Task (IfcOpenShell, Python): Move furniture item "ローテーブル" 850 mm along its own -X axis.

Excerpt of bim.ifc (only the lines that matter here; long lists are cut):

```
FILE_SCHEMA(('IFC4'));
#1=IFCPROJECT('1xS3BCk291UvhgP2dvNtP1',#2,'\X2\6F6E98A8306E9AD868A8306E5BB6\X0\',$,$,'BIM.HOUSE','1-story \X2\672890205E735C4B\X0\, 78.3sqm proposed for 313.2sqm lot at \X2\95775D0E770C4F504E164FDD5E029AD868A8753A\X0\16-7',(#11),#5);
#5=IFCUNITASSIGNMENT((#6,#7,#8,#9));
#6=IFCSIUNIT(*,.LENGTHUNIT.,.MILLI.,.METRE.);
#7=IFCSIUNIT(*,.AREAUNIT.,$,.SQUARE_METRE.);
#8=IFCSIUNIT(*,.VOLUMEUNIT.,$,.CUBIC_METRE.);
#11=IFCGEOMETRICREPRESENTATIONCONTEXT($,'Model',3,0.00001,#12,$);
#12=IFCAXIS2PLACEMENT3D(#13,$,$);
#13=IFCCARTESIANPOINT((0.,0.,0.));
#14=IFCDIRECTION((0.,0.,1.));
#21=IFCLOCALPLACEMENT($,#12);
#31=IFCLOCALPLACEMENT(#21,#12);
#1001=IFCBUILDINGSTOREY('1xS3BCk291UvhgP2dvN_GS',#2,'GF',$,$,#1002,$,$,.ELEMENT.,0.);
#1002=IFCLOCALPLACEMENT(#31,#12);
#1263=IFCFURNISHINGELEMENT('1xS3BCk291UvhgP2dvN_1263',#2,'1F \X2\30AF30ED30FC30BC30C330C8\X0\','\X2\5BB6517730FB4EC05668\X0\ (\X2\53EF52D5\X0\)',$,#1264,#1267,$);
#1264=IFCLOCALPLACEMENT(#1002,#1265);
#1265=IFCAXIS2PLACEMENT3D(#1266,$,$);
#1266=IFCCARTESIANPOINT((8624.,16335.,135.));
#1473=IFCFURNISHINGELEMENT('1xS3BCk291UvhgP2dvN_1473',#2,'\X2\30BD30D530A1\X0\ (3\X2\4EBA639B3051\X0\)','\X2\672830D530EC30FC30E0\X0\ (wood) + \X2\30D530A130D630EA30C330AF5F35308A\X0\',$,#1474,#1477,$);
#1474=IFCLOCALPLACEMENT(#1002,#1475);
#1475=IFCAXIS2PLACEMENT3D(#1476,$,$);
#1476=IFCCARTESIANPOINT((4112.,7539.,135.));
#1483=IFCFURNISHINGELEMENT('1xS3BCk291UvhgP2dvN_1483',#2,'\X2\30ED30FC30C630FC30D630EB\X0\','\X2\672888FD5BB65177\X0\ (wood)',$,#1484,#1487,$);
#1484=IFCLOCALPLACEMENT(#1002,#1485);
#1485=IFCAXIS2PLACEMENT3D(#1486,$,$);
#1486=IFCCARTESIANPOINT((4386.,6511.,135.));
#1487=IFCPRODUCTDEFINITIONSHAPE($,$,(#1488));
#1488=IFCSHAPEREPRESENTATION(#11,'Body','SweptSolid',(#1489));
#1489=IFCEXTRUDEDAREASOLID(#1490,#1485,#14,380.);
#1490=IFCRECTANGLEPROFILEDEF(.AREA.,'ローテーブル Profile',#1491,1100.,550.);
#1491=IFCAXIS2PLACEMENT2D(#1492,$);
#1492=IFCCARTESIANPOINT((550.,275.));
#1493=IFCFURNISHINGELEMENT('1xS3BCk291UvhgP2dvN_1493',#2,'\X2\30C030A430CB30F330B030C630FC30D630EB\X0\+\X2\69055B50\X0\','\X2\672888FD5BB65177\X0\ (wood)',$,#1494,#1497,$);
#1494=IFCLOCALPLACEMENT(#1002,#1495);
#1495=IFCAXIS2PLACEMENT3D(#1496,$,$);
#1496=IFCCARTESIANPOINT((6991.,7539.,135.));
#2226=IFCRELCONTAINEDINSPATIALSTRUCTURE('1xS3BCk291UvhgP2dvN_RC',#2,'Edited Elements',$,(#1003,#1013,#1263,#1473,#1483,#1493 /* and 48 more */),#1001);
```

```python
import ifcopenshell
import ifcopenshell.api.geometry
import ifcopenshell.util.placement

model = ifcopenshell.open("bim.ifc")

item = model.by_guid("1xS3BCk291UvhgP2dvN_1483")
matrix = ifcopenshell.util.placement.get_local_placement(item.ObjectPlacement)
matrix[:3, 3] -= matrix[:3, 0] * 850.0
ifcopenshell.api.geometry.edit_object_placement(model, product=item, matrix=matrix, is_si=False)

print(ifcopenshell.util.placement.get_local_placement(item.ObjectPlacement).round(3) + 0.0)

model.write("bim_rev.ifc")
```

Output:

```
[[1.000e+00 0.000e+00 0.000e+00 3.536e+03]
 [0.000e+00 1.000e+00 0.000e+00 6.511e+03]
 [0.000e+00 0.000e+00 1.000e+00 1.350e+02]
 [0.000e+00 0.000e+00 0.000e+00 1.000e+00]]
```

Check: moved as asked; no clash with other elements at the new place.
